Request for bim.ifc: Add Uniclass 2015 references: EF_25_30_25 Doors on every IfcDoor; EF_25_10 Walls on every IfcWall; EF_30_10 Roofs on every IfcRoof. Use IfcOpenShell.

First a look at what the model holds.

```python
import ifcopenshell

model = ifcopenshell.open("bim.ifc")
print(model.schema)
print("classifications:", [c.Name for c in model.by_type("IfcClassification")])
for ifc_class in ("IfcDoor", "IfcRoof", "IfcStair", "IfcWall", "IfcWindow"):
    print(ifc_class, len(model.by_type(ifc_class)))
```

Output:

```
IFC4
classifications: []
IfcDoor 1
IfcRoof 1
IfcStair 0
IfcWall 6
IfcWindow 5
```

```python
import ifcopenshell
import ifcopenshell.api.classification

model = ifcopenshell.open("bim.ifc")

system = ifcopenshell.api.classification.add_classification(model, classification="Uniclass 2015")

codes = {
    "IfcDoor": ("EF_25_30_25", "Doors"),
    "IfcWall": ("EF_25_10", "Walls"),
    "IfcRoof": ("EF_30_10", "Roofs"),
}
for ifc_class, (code, name) in codes.items():
    products = model.by_type(ifc_class)
    ifcopenshell.api.classification.add_reference(
        model, products=products, classification=system, identification=code, name=name
    )
    print(code, len(products))

model.write("bim_updated.ifc")
```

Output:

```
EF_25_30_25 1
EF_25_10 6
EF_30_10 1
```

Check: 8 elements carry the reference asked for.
